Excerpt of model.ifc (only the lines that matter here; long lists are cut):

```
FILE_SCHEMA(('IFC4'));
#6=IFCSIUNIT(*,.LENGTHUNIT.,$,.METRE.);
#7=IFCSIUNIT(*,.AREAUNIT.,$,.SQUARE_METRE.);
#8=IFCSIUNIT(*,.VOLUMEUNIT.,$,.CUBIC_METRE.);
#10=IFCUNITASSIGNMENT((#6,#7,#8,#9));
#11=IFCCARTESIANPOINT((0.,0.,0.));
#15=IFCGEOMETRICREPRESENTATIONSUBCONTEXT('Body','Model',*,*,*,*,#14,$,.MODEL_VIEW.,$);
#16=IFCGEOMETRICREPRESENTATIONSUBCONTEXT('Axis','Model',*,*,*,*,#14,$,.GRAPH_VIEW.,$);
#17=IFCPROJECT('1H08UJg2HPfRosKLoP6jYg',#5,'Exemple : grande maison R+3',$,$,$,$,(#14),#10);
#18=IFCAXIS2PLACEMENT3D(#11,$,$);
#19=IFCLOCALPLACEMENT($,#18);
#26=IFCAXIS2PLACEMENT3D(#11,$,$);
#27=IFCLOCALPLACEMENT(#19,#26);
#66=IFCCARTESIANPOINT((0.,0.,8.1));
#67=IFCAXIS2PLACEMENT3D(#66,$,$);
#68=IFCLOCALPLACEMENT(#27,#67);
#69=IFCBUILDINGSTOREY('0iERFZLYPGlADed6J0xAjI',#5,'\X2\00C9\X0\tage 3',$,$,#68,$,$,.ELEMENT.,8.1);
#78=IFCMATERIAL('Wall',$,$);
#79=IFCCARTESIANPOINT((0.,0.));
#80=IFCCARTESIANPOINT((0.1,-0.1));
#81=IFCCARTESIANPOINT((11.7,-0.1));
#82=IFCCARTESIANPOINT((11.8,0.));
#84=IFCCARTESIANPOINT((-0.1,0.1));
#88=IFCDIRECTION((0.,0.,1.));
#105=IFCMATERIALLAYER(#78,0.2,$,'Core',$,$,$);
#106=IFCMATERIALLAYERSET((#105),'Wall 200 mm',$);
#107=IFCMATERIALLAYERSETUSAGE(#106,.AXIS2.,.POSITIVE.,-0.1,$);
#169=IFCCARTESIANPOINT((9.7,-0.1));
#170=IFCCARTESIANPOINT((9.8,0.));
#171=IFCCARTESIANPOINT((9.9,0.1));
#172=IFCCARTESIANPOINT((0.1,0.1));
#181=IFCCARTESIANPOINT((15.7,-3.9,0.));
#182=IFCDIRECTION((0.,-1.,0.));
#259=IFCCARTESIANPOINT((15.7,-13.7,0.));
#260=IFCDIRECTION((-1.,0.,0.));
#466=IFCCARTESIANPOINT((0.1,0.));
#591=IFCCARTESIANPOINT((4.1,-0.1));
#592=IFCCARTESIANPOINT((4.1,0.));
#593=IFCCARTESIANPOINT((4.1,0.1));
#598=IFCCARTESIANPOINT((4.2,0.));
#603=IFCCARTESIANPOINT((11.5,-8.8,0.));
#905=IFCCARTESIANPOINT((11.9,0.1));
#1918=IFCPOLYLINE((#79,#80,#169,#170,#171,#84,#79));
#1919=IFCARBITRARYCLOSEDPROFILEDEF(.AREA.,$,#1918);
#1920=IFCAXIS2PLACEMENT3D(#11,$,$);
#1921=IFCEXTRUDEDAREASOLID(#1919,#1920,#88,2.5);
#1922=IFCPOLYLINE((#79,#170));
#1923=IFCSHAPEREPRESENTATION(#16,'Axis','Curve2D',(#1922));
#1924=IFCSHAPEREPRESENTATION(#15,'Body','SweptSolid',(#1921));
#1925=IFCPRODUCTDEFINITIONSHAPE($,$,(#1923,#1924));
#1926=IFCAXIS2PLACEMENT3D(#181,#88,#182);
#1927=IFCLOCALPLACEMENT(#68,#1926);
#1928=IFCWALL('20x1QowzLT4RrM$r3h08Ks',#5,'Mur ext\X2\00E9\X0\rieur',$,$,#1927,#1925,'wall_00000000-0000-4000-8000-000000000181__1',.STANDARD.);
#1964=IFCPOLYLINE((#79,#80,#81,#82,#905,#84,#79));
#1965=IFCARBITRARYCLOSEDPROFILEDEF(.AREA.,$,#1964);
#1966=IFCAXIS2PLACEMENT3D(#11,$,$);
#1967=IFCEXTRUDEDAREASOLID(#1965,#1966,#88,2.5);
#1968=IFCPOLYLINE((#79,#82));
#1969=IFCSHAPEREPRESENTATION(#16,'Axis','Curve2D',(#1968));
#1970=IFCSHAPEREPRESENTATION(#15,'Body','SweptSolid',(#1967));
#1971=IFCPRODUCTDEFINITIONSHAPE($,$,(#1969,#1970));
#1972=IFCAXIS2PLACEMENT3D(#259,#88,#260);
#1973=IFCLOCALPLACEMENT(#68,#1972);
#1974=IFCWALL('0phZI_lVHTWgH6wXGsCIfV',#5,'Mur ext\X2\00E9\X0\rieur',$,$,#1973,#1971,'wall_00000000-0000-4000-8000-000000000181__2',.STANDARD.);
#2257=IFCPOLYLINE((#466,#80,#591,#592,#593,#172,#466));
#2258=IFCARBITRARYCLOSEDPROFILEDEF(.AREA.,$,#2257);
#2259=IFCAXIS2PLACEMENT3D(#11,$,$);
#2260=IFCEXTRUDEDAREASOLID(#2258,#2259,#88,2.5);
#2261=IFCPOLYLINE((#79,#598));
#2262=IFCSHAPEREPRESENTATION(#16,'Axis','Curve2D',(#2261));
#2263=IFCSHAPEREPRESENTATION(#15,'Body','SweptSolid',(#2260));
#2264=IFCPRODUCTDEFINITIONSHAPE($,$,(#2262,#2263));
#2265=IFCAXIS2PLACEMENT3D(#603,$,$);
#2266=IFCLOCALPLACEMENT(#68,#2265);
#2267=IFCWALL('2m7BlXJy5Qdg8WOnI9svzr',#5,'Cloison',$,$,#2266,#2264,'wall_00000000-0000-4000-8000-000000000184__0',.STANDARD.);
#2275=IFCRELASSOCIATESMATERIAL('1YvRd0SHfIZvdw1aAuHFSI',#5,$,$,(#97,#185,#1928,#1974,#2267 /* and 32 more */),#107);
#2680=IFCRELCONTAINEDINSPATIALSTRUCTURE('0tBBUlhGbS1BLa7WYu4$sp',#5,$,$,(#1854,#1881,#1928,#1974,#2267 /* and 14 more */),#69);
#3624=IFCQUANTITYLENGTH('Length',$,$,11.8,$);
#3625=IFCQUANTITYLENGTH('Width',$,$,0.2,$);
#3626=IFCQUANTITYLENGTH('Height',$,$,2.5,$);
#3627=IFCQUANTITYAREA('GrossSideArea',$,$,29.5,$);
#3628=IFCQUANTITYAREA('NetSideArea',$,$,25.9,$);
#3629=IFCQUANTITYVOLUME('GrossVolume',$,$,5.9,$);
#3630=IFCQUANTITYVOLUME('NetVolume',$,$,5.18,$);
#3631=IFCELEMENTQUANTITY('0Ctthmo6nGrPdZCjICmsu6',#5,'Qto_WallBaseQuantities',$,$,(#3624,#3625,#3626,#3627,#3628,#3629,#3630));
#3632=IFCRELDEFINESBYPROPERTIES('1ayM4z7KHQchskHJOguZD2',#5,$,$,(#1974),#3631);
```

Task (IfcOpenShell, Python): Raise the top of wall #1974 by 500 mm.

```python
import ifcopenshell
import ifcopenshell.api.pset
import ifcopenshell.geom
import ifcopenshell.util.element
import ifcopenshell.util.representation
import ifcopenshell.util.shape
import ifcopenshell.util.unit

model = ifcopenshell.open("model.ifc")
unit_scale = ifcopenshell.util.unit.calculate_unit_scale(model)
area_scale = ifcopenshell.util.unit.calculate_unit_scale(model, "AREAUNIT")
volume_scale = ifcopenshell.util.unit.calculate_unit_scale(model, "VOLUMEUNIT")
settings = ifcopenshell.geom.settings()


def volume(element):
    """Net volume in cubic metres, openings subtracted."""
    shape = ifcopenshell.geom.create_shape(settings, element)
    return ifcopenshell.util.shape.get_volume(shape.geometry)


wall = model.by_guid("0phZI_lVHTWgH6wXGsCIfV")
before = volume(wall)

body = ifcopenshell.util.representation.get_representation(wall, "Model", "Body")
solid = body.Items[0]
old_height = solid.Depth
solid.Depth += 0.5
after = volume(wall)
thickness = 0.2  # wall thickness in metres

# Update the stored height, areas and volumes.
qto = model.by_id(ifcopenshell.util.element.get_pset(wall, "Qto_WallBaseQuantities", should_inherit=False)["id"])
ifcopenshell.api.pset.edit_qto(model, qto=qto, properties={
    "Height": solid.Depth,
    "GrossSideArea": ifcopenshell.util.element.get_pset(wall, "Qto_WallBaseQuantities", "GrossSideArea") * solid.Depth / old_height,
    "NetSideArea": after / thickness / area_scale,
    "GrossVolume": ifcopenshell.util.element.get_pset(wall, "Qto_WallBaseQuantities", "GrossVolume") * solid.Depth / old_height,
    "NetVolume": after / volume_scale,
})

print(f"height {old_height:g} -> {solid.Depth:g}, volume {before:.3f} -> {after:.3f} m3")

model.write("model_rev.ifc")
```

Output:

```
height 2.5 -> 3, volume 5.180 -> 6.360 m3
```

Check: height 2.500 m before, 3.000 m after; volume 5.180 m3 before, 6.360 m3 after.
